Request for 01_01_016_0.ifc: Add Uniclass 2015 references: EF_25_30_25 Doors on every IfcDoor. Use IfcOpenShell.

First a look at what the model holds.

```python
import ifcopenshell

model = ifcopenshell.open("01_01_016_0.ifc")
print(model.schema)
print("classifications:", [c.Name for c in model.by_type("IfcClassification")])
for ifc_class in ("IfcDoor", "IfcRoof", "IfcStair", "IfcWall", "IfcWindow"):
    print(ifc_class, len(model.by_type(ifc_class)))
```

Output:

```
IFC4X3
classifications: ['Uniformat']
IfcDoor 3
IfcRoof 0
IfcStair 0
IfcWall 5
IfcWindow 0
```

```python
import ifcopenshell
import ifcopenshell.api.classification

model = ifcopenshell.open("01_01_016_0.ifc")

system = ifcopenshell.api.classification.add_classification(model, classification="Uniclass 2015")

codes = {
    "IfcDoor": ("EF_25_30_25", "Doors"),
}
for ifc_class, (code, name) in codes.items():
    products = model.by_type(ifc_class)
    ifcopenshell.api.classification.add_reference(
        model, products=products, classification=system, identification=code, name=name
    )
    print(code, len(products))

model.write("01_01_016_0-out.ifc")
```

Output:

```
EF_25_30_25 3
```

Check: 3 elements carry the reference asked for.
